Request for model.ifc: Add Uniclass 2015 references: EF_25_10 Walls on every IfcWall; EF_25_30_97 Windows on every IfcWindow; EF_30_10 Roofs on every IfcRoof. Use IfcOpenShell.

First a look at what the model holds.

```python
import ifcopenshell

model = ifcopenshell.open("model.ifc")
print(model.schema)
print("classifications:", [c.Name for c in model.by_type("IfcClassification")])
for ifc_class in ("IfcDoor", "IfcRoof", "IfcStair", "IfcWall", "IfcWindow"):
    print(ifc_class, len(model.by_type(ifc_class)))
```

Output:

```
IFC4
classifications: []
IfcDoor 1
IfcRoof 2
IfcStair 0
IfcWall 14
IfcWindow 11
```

```python
import ifcopenshell
import ifcopenshell.api.classification

model = ifcopenshell.open("model.ifc")

system = ifcopenshell.api.classification.add_classification(model, classification="Uniclass 2015")

codes = {
    "IfcWall": ("EF_25_10", "Walls"),
    "IfcWindow": ("EF_25_30_97", "Windows"),
    "IfcRoof": ("EF_30_10", "Roofs"),
}
for ifc_class, (code, name) in codes.items():
    products = model.by_type(ifc_class)
    ifcopenshell.api.classification.add_reference(
        model, products=products, classification=system, identification=code, name=name
    )
    print(code, len(products))

model.write("model_updated.ifc")
```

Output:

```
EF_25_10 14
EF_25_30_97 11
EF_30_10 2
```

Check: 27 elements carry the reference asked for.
